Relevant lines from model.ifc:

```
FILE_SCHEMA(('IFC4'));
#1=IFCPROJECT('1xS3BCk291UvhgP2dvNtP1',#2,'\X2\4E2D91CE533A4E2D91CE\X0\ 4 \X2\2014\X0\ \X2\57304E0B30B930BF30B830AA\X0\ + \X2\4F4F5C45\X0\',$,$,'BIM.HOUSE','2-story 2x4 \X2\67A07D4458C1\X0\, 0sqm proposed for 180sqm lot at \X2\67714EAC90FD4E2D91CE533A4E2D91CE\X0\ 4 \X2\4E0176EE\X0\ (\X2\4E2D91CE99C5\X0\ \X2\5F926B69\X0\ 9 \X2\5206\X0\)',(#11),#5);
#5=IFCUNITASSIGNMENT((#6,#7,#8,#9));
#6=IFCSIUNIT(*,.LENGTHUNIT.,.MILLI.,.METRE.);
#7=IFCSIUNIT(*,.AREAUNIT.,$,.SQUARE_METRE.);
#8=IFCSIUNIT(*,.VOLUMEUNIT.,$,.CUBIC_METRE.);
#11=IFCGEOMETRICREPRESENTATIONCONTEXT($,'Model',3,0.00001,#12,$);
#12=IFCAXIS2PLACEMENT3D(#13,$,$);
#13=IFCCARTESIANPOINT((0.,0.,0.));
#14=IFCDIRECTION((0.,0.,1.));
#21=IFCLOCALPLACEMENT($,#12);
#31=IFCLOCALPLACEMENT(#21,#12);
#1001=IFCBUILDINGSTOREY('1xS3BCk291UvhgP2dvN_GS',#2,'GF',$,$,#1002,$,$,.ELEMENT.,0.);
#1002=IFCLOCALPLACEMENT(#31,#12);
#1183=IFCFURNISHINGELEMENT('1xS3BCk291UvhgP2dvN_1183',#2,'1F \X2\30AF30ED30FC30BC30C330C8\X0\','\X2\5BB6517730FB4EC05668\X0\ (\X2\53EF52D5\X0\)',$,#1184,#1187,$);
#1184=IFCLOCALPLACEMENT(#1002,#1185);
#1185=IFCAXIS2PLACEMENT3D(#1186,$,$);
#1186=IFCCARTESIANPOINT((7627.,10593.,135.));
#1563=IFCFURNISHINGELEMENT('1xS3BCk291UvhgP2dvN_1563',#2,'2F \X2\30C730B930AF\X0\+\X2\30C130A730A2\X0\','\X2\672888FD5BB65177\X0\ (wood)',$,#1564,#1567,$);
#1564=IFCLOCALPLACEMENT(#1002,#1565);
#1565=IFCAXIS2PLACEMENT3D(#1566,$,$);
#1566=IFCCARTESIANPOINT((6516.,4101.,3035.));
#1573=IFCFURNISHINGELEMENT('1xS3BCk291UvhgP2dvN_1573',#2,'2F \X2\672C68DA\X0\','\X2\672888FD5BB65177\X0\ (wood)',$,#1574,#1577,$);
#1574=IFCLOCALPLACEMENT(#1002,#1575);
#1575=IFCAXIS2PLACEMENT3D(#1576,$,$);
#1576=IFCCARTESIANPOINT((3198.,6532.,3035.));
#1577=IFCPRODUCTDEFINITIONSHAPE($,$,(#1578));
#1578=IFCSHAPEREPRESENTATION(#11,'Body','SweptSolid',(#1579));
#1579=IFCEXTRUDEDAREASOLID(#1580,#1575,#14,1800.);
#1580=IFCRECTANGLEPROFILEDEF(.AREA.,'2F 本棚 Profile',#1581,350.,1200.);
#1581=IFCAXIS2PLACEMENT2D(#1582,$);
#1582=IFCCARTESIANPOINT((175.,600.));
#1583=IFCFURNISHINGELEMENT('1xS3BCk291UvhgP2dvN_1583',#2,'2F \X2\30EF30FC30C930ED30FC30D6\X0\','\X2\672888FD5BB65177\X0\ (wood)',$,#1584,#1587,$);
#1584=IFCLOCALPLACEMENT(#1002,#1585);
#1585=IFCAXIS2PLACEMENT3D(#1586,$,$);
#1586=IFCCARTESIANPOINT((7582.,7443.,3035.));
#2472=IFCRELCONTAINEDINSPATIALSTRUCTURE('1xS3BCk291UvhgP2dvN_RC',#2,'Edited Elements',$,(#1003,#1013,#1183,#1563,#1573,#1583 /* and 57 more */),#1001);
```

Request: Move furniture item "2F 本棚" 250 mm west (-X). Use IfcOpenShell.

```python
import ifcopenshell
import ifcopenshell.api.geometry
import ifcopenshell.util.placement
import ifcopenshell.util.unit

model = ifcopenshell.open("model.ifc")
unit_scale = ifcopenshell.util.unit.calculate_unit_scale(model)

item = model.by_id(1573)
matrix = ifcopenshell.util.placement.get_local_placement(item.ObjectPlacement)
matrix[0, 3] -= 0.25 / unit_scale
ifcopenshell.api.geometry.edit_object_placement(model, product=item, matrix=matrix, is_si=False)

print(ifcopenshell.util.placement.get_local_placement(item.ObjectPlacement).round(3) + 0.0)

model.write("model-out.ifc")
```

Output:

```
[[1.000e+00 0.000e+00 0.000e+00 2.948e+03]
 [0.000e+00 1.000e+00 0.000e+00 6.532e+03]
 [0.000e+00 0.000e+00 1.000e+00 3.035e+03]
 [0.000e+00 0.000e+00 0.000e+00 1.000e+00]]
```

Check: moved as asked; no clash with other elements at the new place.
